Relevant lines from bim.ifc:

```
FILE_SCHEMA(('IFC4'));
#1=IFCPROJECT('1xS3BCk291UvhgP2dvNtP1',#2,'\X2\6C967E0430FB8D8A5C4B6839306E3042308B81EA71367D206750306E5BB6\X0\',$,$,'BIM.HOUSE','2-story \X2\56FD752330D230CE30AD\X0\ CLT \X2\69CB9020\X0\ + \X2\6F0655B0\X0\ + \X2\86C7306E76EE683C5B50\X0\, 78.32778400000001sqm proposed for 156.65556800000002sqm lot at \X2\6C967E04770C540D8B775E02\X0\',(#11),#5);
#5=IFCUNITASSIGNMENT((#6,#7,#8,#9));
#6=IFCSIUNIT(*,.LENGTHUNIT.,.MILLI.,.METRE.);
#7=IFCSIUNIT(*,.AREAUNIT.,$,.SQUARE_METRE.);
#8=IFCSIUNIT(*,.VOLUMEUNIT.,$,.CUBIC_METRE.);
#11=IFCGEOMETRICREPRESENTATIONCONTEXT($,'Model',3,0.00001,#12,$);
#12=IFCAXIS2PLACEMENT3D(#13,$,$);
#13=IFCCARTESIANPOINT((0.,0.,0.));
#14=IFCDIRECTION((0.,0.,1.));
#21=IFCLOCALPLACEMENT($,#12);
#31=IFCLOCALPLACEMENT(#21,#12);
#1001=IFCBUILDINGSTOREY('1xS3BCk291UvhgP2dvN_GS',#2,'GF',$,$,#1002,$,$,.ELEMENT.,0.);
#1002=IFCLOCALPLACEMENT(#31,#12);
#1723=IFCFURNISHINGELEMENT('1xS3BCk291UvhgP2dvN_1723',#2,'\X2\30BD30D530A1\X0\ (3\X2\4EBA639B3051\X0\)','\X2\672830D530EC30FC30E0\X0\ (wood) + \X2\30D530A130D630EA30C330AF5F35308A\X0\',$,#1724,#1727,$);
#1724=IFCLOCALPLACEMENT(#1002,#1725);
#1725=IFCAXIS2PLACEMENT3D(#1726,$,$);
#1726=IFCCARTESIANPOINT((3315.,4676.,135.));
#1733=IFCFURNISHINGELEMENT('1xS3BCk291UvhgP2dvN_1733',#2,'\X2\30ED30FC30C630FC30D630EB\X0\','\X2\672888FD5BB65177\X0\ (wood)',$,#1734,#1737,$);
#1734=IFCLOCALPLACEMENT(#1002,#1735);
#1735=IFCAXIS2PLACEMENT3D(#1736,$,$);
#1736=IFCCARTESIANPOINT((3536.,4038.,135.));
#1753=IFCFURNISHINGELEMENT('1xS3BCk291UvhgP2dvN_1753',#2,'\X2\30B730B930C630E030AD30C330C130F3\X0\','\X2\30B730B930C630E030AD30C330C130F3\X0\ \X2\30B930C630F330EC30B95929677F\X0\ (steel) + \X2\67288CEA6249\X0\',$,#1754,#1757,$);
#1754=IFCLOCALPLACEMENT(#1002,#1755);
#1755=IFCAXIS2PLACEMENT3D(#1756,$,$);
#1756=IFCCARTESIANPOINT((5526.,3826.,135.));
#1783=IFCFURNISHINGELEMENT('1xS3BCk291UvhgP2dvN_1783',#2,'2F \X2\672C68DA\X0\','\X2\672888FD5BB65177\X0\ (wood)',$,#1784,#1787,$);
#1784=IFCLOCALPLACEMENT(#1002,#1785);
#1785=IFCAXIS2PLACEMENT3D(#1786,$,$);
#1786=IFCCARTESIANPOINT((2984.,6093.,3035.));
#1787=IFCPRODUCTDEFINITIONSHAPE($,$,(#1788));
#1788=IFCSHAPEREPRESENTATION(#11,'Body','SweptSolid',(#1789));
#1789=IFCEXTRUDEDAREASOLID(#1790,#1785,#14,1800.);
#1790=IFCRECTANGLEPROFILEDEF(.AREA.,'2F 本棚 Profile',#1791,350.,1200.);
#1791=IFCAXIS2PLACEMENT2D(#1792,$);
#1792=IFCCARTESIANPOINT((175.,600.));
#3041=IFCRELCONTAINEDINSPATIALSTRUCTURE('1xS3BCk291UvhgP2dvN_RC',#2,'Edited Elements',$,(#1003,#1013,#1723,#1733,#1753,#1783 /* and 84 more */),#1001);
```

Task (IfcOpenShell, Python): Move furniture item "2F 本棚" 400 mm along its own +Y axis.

```python
import ifcopenshell
import ifcopenshell.api.geometry
import ifcopenshell.util.placement

model = ifcopenshell.open("bim.ifc")

item = model.by_id(1783)
matrix = ifcopenshell.util.placement.get_local_placement(item.ObjectPlacement)
matrix[:3, 3] += matrix[:3, 1] * 400.0
ifcopenshell.api.geometry.edit_object_placement(model, product=item, matrix=matrix, is_si=False)

print(ifcopenshell.util.placement.get_local_placement(item.ObjectPlacement).round(3) + 0.0)

model.write("bim_v2.ifc")
```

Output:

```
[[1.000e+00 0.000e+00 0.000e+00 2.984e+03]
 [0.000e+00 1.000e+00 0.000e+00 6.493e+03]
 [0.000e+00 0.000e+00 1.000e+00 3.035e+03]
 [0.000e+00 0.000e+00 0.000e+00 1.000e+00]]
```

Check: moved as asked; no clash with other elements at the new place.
